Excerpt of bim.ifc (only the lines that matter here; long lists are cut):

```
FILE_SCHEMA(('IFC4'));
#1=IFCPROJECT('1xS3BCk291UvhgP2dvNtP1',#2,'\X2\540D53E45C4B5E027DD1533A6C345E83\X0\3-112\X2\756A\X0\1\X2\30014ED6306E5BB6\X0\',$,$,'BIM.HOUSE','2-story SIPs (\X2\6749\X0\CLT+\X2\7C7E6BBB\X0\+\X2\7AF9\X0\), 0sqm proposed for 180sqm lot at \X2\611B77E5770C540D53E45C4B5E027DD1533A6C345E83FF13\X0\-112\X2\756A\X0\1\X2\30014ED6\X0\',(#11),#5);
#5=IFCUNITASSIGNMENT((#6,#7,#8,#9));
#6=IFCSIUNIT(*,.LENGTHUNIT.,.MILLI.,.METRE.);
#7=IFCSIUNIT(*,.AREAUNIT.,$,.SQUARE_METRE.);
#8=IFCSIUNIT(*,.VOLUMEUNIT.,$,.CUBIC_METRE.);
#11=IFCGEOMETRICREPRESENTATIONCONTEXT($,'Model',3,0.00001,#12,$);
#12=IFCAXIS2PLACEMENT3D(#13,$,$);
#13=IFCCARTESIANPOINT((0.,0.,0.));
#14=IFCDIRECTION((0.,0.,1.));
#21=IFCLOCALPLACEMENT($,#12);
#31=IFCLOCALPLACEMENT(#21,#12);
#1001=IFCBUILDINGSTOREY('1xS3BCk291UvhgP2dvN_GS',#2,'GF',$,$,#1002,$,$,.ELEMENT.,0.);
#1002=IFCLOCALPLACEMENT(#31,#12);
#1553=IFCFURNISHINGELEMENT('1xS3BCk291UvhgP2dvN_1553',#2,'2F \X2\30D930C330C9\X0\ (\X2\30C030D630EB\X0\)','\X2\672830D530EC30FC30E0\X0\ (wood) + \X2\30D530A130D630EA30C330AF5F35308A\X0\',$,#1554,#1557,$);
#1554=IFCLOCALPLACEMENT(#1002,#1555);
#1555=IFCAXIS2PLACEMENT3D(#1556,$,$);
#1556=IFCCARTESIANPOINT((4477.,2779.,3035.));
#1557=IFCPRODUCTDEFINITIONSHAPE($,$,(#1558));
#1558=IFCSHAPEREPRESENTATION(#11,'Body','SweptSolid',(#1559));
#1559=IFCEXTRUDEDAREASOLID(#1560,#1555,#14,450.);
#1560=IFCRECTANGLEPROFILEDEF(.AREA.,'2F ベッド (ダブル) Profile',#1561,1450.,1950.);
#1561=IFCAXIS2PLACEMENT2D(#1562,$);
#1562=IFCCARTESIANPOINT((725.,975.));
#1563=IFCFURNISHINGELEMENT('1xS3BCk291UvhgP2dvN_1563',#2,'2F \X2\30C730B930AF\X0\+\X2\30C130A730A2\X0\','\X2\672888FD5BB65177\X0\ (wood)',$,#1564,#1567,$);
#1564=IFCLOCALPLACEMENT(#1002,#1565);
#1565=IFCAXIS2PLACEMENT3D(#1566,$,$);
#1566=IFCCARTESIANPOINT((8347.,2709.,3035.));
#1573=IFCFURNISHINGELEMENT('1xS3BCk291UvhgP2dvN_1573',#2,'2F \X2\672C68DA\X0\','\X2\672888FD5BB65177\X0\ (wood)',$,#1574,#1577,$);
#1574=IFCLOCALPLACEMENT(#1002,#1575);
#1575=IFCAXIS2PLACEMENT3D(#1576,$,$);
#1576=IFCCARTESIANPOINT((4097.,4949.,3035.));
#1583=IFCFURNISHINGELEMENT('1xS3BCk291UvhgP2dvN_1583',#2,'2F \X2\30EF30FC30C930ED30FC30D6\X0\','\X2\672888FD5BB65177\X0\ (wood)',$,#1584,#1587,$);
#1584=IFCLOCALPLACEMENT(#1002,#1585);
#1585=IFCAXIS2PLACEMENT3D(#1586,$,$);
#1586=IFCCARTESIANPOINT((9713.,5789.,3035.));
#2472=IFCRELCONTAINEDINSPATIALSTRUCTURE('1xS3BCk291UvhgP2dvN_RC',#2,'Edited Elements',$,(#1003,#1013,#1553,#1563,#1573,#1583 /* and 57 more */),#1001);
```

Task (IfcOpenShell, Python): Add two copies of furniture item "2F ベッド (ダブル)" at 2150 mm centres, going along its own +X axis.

```python
import ifcopenshell
import ifcopenshell.api.geometry
import ifcopenshell.api.root
import ifcopenshell.util.element
import ifcopenshell.util.placement
import ifcopenshell.util.unit

model = ifcopenshell.open("bim.ifc")
unit_scale = ifcopenshell.util.unit.calculate_unit_scale(model)


def reuse_history(source, copy):
    """copy_class also copies each property set's owner history, people and application; keep the originals."""
    for rel in copy.IsDefinedBy:
        if rel.is_a("IfcRelDefinesByProperties") and (history := rel.RelatingPropertyDefinition.OwnerHistory):
            rel.RelatingPropertyDefinition.OwnerHistory = source.OwnerHistory
            ifcopenshell.util.element.remove_deep2(model, history)


source = model.by_guid("1xS3BCk291UvhgP2dvN_1553")
base = ifcopenshell.util.placement.get_local_placement(source.ObjectPlacement)
step = base[:3, 0] * 2.15 / unit_scale

for i in range(1, 3):
    copy = ifcopenshell.api.root.copy_class(model, product=source)
    copy.Representation = ifcopenshell.util.element.copy_deep(
        model, source.Representation, exclude=["IfcGeometricRepresentationContext", "IfcRepresentationMap"]
    )
    reuse_history(source, copy)
    matrix = base.copy()
    matrix[:3, 3] += i * step
    print("added at", matrix[:3, 3].round(3) + 0.0)
    ifcopenshell.api.geometry.edit_object_placement(model, product=copy, matrix=matrix, is_si=False)

model.write("bim-out.ifc")
```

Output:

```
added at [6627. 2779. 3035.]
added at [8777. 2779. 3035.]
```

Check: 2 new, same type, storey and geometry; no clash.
